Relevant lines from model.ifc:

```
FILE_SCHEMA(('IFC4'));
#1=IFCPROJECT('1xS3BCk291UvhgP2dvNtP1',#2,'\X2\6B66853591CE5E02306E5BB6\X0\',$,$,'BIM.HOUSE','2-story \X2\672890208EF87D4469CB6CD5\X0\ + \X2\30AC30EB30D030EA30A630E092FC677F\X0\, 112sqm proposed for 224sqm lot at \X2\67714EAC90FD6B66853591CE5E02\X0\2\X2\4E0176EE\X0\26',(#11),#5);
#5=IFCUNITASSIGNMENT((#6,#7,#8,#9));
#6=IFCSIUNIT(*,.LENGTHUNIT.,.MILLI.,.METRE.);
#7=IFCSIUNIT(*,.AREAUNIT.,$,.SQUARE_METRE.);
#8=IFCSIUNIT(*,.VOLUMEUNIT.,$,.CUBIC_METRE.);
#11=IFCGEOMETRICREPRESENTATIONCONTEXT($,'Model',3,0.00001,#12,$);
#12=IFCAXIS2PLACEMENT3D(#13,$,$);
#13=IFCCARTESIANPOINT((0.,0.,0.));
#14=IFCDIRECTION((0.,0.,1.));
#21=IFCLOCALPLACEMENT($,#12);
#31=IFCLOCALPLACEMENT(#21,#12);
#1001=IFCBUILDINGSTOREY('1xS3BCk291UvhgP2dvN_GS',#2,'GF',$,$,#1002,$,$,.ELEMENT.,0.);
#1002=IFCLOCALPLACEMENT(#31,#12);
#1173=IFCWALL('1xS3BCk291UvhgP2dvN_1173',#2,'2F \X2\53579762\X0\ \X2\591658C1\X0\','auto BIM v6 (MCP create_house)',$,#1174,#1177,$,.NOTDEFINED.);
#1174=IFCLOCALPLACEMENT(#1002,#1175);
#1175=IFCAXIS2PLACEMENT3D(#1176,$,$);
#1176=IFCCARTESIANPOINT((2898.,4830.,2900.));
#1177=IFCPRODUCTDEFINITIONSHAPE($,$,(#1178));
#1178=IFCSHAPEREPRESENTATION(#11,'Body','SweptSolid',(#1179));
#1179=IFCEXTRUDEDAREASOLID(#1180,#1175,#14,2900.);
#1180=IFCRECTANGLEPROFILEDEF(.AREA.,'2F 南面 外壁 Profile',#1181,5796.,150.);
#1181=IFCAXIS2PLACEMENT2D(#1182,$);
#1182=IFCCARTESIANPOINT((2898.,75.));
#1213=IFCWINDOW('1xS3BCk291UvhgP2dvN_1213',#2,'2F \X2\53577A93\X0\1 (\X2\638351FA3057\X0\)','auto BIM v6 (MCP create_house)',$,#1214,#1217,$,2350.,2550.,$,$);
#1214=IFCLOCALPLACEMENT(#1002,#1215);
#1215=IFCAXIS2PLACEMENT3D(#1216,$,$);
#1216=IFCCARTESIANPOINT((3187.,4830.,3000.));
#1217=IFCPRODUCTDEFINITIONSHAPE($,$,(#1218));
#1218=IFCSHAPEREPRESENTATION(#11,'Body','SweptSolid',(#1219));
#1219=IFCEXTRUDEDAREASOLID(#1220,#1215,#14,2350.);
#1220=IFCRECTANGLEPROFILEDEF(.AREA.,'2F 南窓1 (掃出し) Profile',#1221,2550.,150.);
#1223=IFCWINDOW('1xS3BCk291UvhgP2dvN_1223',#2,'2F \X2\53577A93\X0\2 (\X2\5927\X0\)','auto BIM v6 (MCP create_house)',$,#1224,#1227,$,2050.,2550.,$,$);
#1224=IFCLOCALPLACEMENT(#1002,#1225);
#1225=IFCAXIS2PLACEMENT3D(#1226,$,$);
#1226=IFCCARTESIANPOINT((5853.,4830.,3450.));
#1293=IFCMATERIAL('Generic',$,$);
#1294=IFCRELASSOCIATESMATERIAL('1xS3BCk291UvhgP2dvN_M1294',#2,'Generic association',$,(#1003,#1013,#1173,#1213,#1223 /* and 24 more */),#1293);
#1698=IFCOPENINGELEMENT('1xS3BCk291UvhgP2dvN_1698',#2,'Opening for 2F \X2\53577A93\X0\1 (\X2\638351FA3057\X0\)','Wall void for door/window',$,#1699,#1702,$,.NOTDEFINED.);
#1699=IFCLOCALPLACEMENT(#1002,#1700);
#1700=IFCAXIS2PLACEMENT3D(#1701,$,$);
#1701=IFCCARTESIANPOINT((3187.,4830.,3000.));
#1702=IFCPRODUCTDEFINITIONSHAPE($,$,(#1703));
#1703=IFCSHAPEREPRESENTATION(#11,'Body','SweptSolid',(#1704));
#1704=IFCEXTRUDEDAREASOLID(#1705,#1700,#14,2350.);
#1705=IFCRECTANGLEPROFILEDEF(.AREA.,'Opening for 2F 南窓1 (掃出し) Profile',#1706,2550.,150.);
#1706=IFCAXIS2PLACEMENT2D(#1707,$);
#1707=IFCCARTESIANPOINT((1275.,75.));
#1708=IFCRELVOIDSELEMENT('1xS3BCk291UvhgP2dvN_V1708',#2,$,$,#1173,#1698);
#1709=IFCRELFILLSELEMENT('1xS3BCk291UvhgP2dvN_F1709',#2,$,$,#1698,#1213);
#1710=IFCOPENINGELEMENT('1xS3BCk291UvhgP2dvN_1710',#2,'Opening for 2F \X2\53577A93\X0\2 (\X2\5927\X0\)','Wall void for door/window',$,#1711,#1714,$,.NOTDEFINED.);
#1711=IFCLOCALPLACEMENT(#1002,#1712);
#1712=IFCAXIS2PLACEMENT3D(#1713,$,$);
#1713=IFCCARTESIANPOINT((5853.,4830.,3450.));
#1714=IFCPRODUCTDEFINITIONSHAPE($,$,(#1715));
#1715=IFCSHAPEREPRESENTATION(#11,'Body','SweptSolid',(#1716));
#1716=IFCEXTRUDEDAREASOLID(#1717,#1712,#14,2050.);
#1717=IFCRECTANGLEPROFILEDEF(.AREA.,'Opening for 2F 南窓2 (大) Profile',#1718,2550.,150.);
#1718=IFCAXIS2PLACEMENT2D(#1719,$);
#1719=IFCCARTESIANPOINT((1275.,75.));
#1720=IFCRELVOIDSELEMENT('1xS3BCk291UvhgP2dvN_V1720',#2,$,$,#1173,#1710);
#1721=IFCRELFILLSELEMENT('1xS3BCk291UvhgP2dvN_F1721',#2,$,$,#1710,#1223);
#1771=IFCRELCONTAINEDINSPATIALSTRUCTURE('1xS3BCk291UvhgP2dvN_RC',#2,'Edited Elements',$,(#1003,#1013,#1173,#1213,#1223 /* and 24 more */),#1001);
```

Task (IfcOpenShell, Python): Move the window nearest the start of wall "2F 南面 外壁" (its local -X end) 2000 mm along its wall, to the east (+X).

```python
import ifcopenshell
import ifcopenshell.api.geometry
import ifcopenshell.util.placement
import ifcopenshell.util.unit

model = ifcopenshell.open("model.ifc")
unit_scale = ifcopenshell.util.unit.calculate_unit_scale(model)

window = model.by_id(1213)
opening = window.FillsVoids[0].RelatingOpeningElement
wall = opening.VoidsElements[0].RelatingBuildingElement

wall_matrix = ifcopenshell.util.placement.get_local_placement(wall.ObjectPlacement)
shift = wall_matrix[:3, 0] * 2 / unit_scale
before = ifcopenshell.util.placement.get_local_placement(window.ObjectPlacement)[:3, 3].copy()

# The window is not placed relative to its opening, so move both.
for product in (opening, window):
    matrix = ifcopenshell.util.placement.get_local_placement(product.ObjectPlacement)
    matrix[:3, 3] += shift
    ifcopenshell.api.geometry.edit_object_placement(model, product=product, matrix=matrix, is_si=False)

after = ifcopenshell.util.placement.get_local_placement(window.ObjectPlacement)[:3, 3]
print("window moved by", (after - before).round(3) + 0.0)

model.write("model_rev.ifc")
```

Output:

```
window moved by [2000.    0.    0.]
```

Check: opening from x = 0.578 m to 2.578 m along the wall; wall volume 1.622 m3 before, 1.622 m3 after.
